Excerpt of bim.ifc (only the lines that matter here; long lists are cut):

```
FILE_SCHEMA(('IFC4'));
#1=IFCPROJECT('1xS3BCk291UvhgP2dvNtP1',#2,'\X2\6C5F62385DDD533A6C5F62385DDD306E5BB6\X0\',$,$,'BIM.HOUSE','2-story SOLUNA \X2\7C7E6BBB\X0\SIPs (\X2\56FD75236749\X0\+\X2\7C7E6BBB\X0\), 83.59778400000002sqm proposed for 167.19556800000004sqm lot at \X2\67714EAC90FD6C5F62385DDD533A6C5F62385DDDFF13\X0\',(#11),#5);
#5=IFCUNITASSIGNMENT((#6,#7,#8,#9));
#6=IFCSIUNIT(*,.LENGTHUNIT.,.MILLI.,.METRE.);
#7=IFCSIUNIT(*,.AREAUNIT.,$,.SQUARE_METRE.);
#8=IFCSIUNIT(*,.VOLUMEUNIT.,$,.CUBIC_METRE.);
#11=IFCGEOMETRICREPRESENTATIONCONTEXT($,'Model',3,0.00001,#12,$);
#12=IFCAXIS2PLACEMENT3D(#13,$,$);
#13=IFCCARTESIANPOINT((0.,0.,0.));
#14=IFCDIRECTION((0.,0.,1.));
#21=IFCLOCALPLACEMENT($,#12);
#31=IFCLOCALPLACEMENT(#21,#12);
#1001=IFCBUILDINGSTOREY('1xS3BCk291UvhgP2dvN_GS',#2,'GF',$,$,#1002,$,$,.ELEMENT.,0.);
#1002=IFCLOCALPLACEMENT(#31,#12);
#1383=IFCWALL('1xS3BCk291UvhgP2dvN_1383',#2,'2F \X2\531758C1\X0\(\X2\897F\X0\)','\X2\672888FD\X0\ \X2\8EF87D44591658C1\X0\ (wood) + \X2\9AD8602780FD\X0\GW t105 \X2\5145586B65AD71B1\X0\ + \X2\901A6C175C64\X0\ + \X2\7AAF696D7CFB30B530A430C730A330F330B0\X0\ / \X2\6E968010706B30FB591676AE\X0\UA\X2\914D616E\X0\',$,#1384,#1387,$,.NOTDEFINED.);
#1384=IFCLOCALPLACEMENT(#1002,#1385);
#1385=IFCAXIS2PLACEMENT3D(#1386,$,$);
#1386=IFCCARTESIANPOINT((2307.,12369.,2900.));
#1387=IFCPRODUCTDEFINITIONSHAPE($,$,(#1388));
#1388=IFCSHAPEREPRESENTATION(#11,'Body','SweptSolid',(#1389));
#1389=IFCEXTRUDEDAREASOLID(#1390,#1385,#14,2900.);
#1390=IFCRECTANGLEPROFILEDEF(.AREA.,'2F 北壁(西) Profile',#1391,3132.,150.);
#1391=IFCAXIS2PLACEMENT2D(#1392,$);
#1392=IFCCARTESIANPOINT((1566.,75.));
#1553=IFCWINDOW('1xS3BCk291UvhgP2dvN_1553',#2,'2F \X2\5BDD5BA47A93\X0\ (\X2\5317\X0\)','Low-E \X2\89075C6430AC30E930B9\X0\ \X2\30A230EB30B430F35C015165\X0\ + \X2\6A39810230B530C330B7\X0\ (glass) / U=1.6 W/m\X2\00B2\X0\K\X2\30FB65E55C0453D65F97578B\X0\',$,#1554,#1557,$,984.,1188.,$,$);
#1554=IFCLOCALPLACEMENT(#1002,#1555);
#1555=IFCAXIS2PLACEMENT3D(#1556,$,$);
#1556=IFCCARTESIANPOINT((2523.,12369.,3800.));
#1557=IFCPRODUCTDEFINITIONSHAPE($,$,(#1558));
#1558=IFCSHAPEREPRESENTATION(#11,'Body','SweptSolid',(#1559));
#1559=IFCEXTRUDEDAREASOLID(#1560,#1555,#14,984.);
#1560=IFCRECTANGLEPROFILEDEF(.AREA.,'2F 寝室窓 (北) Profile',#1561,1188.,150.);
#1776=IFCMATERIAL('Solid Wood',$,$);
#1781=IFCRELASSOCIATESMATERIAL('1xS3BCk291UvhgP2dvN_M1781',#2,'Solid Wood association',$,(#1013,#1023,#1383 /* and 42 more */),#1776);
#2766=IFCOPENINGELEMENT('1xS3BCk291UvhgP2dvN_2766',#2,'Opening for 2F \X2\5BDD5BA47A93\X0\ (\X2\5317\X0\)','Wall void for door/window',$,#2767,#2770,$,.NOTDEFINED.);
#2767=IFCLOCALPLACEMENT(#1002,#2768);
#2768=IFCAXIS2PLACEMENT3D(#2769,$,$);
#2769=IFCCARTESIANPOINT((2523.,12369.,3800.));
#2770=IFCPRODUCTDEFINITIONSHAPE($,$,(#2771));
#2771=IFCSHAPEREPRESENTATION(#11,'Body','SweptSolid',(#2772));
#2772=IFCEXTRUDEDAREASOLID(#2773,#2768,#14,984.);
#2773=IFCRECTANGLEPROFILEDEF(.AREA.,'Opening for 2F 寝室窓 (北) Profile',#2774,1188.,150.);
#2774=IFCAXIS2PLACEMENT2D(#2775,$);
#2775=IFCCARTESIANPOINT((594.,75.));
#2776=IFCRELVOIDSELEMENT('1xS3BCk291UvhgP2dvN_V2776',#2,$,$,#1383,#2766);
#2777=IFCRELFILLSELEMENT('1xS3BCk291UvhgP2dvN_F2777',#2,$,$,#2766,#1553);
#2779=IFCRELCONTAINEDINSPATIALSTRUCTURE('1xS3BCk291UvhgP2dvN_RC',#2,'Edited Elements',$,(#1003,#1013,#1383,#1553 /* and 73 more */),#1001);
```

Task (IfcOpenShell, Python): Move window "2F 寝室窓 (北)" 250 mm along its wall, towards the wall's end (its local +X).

```python
import ifcopenshell
import ifcopenshell.api.geometry
import ifcopenshell.util.placement
import ifcopenshell.util.unit

model = ifcopenshell.open("bim.ifc")
unit_scale = ifcopenshell.util.unit.calculate_unit_scale(model)

window = model.by_guid("1xS3BCk291UvhgP2dvN_1553")
opening = window.FillsVoids[0].RelatingOpeningElement
wall = opening.VoidsElements[0].RelatingBuildingElement

wall_matrix = ifcopenshell.util.placement.get_local_placement(wall.ObjectPlacement)
shift = wall_matrix[:3, 0] * 0.25 / unit_scale
before = ifcopenshell.util.placement.get_local_placement(window.ObjectPlacement)[:3, 3].copy()

# The window is not placed relative to its opening, so move both.
for product in (opening, window):
    matrix = ifcopenshell.util.placement.get_local_placement(product.ObjectPlacement)
    matrix[:3, 3] += shift
    ifcopenshell.api.geometry.edit_object_placement(model, product=product, matrix=matrix, is_si=False)

after = ifcopenshell.util.placement.get_local_placement(window.ObjectPlacement)[:3, 3]
print("window moved by", (after - before).round(3) + 0.0)

model.write("bim-out.ifc")
```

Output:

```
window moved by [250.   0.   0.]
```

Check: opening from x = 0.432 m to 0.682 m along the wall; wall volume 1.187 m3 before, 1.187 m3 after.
